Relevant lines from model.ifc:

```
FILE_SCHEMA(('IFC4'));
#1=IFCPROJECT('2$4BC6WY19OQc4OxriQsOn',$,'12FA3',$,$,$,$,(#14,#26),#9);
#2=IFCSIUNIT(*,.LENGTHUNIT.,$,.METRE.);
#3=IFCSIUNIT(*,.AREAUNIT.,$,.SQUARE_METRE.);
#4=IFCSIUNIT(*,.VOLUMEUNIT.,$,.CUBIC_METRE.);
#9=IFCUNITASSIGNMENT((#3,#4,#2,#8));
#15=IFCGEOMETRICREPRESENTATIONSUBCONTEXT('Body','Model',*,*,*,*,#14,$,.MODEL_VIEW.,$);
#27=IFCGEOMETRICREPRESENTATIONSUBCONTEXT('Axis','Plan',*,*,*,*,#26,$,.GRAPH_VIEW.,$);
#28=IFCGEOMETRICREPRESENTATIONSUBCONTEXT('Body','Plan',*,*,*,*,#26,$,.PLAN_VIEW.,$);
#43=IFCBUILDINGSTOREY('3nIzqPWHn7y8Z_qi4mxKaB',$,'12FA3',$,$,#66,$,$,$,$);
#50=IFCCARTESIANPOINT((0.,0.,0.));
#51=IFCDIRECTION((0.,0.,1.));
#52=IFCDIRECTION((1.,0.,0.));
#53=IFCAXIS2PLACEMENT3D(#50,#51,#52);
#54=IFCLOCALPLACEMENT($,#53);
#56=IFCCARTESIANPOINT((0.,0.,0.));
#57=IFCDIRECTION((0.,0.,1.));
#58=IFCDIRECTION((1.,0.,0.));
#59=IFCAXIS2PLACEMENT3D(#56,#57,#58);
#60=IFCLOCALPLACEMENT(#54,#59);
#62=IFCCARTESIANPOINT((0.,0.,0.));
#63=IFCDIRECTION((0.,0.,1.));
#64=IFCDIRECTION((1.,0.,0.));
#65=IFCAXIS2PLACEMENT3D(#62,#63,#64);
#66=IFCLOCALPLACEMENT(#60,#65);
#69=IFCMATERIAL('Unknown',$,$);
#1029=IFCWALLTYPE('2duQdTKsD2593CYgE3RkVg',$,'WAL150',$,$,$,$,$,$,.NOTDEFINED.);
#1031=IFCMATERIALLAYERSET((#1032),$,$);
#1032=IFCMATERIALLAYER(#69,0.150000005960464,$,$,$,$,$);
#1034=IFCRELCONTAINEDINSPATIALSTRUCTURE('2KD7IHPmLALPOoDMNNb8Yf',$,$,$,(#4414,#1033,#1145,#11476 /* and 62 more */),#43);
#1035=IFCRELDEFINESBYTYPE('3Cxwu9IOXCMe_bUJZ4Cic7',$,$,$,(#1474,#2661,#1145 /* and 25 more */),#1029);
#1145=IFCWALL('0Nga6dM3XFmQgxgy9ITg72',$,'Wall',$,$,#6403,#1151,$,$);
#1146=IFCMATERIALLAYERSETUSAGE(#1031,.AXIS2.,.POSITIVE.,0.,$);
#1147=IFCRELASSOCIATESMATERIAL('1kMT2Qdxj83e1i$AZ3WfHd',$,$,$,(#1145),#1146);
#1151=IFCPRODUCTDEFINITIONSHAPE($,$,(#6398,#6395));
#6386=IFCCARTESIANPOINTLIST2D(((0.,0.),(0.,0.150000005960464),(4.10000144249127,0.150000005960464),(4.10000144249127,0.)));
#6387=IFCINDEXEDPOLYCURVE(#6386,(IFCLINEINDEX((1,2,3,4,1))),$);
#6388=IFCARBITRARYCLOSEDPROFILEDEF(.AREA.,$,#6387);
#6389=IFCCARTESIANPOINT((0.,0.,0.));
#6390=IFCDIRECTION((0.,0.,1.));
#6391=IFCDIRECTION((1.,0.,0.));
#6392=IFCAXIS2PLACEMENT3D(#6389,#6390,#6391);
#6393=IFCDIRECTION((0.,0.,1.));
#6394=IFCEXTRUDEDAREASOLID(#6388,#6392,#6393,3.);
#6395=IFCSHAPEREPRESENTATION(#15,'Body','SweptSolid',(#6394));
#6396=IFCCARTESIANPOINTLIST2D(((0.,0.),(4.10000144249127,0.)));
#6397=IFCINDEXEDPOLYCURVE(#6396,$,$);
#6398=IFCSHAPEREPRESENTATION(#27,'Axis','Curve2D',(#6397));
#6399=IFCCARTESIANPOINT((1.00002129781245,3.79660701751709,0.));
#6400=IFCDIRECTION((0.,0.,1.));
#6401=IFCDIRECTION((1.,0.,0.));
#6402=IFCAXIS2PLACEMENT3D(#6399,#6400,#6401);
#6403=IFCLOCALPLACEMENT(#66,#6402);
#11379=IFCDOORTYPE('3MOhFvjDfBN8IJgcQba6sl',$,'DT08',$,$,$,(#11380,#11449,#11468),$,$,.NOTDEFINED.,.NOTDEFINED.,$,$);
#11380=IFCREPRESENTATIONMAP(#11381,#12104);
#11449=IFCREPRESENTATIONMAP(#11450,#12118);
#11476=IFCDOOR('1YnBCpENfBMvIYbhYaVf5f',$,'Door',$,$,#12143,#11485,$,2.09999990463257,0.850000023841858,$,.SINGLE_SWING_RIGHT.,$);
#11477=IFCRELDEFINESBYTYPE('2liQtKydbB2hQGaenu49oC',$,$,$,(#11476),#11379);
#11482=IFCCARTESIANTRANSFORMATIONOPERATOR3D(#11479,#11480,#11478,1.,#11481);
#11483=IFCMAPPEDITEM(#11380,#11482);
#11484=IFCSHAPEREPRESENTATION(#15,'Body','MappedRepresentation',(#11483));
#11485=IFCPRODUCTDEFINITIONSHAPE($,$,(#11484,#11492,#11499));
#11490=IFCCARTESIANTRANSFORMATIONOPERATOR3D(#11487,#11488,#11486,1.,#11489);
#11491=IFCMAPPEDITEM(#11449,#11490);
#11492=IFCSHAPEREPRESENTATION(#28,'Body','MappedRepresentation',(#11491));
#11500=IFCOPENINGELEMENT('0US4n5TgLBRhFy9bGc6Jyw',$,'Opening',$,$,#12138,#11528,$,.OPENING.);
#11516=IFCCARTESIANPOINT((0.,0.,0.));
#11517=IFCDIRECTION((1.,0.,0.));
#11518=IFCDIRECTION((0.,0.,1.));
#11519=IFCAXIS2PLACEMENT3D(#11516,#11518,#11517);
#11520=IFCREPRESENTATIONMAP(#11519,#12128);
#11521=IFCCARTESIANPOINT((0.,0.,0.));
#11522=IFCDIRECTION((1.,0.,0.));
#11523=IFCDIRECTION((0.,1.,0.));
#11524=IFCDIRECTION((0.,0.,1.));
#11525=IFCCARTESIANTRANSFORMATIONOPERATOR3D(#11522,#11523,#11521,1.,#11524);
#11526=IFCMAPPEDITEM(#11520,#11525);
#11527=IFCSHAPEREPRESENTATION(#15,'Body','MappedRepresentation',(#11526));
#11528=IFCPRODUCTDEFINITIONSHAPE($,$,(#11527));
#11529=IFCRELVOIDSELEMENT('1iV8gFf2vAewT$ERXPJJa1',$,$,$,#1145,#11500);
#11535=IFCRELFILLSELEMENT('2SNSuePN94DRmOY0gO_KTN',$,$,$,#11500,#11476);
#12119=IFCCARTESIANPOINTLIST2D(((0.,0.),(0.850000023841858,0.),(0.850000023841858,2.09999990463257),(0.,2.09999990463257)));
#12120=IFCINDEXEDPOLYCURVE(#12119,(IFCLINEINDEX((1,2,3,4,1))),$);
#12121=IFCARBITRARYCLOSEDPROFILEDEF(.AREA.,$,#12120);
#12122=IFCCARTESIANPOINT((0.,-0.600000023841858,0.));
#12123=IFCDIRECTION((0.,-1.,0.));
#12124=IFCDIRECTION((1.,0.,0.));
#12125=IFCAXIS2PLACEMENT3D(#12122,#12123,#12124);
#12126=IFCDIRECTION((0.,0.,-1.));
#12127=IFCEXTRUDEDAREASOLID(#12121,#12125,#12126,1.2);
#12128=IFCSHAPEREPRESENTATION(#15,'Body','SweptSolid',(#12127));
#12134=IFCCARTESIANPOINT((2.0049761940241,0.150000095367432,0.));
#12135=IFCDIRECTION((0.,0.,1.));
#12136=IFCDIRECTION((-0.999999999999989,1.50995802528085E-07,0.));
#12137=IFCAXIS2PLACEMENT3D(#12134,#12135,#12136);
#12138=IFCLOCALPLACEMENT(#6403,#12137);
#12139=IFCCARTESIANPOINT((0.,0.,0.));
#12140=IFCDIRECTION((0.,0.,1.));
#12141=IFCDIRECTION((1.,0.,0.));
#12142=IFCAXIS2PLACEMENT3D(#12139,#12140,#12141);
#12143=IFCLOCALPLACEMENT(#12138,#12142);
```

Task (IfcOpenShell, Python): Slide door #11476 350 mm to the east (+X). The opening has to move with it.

```python
import ifcopenshell
import ifcopenshell.api.geometry
import ifcopenshell.util.placement
import ifcopenshell.util.unit

model = ifcopenshell.open("model.ifc")
unit_scale = ifcopenshell.util.unit.calculate_unit_scale(model)

door = model.by_id(11476)
opening = door.FillsVoids[0].RelatingOpeningElement
wall = opening.VoidsElements[0].RelatingBuildingElement

wall_matrix = ifcopenshell.util.placement.get_local_placement(wall.ObjectPlacement)
shift = wall_matrix[:3, 0] * 0.35 / unit_scale
before = ifcopenshell.util.placement.get_local_placement(door.ObjectPlacement)[:3, 3].copy()

# The door is placed relative to its opening, so it follows when the opening moves.
matrix = ifcopenshell.util.placement.get_local_placement(opening.ObjectPlacement)
matrix[:3, 3] += shift
ifcopenshell.api.geometry.edit_object_placement(
    model, product=opening, matrix=matrix, is_si=False, should_transform_children=True
)

after = ifcopenshell.util.placement.get_local_placement(door.ObjectPlacement)[:3, 3]
print("door moved by", (after - before).round(3) + 0.0)

model.write("model_edited.ifc")
```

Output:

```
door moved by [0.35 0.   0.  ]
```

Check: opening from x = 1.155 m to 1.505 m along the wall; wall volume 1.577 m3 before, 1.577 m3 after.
